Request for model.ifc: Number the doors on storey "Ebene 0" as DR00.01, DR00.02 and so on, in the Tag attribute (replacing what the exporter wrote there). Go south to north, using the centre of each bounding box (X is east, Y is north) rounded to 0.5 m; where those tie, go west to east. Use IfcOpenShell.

First a look at what the model holds.

```python
import ifcopenshell
import ifcopenshell.util.element
import ifcopenshell.util.placement

model = ifcopenshell.open("model.ifc")
print(model.schema)
storey = next(s for s in model.by_type("IfcBuildingStorey") if s.Name == "Ebene 0")
doors = [e for e in ifcopenshell.util.element.get_decomposition(storey) if e.is_a("IfcDoor")]
for e in sorted(doors, key=lambda e: e.id()):
    origin = ifcopenshell.util.placement.get_local_placement(e.ObjectPlacement)[:3, 3]
    print(e.id(), e.Tag, e.Name, origin.round(2) + 0.0, sep=" | ")
```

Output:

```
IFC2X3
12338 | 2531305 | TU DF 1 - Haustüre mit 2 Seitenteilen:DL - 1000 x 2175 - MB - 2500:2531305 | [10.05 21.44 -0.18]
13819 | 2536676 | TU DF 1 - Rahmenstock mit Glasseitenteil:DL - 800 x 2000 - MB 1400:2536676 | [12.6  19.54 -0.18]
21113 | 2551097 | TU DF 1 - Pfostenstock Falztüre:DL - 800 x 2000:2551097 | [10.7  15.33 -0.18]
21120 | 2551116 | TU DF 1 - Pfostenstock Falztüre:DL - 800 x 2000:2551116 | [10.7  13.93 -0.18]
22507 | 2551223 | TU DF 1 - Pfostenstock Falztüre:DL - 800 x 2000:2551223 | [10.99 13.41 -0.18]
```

```python
import ifcopenshell
import ifcopenshell.geom
import ifcopenshell.util.element
import ifcopenshell.util.shape

model = ifcopenshell.open("model.ifc")
settings = ifcopenshell.geom.settings()
settings.set("use-world-coords", True)


def centre(element):
    shape = ifcopenshell.geom.create_shape(settings, element)
    return ifcopenshell.util.shape.get_bbox_centroid(shape.geometry)


storey = next(s for s in model.by_type("IfcBuildingStorey") if s.Name == "Ebene 0")
doors = [e for e in ifcopenshell.util.element.get_decomposition(storey) if e.is_a("IfcDoor")]

# Insertion points can sit at a corner or the storey origin, so sort by the geometry (in metres).
centres = {e: centre(e) for e in doors}
doors.sort(key=lambda e: (round(centres[e][1] / 0.5), centres[e][0]))

for i, e in enumerate(doors, start=1):
    number = f"DR00.{i:02d}"
    e.Tag = number
    print(e.id(), number)

model.write("model_updated.ifc")
```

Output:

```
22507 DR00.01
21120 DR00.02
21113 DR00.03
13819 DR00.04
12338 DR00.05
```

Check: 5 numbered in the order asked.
